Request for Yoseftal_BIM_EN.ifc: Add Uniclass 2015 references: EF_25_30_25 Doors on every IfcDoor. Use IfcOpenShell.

First a look at what the model holds.

```python
import ifcopenshell

model = ifcopenshell.open("Yoseftal_BIM_EN.ifc")
print(model.schema)
print("classifications:", [c.Name for c in model.by_type("IfcClassification")])
for ifc_class in ("IfcDoor", "IfcRoof", "IfcStair", "IfcWall", "IfcWindow"):
    print(ifc_class, len(model.by_type(ifc_class)))
```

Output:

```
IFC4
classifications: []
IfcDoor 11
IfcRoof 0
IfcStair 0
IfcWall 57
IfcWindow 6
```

```python
import ifcopenshell
import ifcopenshell.api.classification

model = ifcopenshell.open("Yoseftal_BIM_EN.ifc")

system = ifcopenshell.api.classification.add_classification(model, classification="Uniclass 2015")

codes = {
    "IfcDoor": ("EF_25_30_25", "Doors"),
}
for ifc_class, (code, name) in codes.items():
    products = model.by_type(ifc_class)
    ifcopenshell.api.classification.add_reference(
        model, products=products, classification=system, identification=code, name=name
    )
    print(code, len(products))

model.write("Yoseftal_BIM_EN_updated.ifc")
```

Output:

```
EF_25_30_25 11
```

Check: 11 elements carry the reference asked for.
